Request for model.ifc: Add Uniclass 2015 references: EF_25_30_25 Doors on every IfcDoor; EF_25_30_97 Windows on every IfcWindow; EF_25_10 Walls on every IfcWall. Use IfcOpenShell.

First a look at what the model holds.

```python
import ifcopenshell

model = ifcopenshell.open("model.ifc")
print(model.schema)
print("classifications:", [c.Name for c in model.by_type("IfcClassification")])
for ifc_class in ("IfcDoor", "IfcRoof", "IfcStair", "IfcWall", "IfcWindow"):
    print(ifc_class, len(model.by_type(ifc_class)))
```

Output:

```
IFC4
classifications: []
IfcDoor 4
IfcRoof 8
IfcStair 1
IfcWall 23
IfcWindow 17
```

```python
import ifcopenshell
import ifcopenshell.api.classification

model = ifcopenshell.open("model.ifc")

system = ifcopenshell.api.classification.add_classification(model, classification="Uniclass 2015")

codes = {
    "IfcDoor": ("EF_25_30_25", "Doors"),
    "IfcWindow": ("EF_25_30_97", "Windows"),
    "IfcWall": ("EF_25_10", "Walls"),
}
for ifc_class, (code, name) in codes.items():
    products = model.by_type(ifc_class)
    ifcopenshell.api.classification.add_reference(
        model, products=products, classification=system, identification=code, name=name
    )
    print(code, len(products))

model.write("model_updated.ifc")
```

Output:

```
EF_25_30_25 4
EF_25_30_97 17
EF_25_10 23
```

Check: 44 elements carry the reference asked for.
